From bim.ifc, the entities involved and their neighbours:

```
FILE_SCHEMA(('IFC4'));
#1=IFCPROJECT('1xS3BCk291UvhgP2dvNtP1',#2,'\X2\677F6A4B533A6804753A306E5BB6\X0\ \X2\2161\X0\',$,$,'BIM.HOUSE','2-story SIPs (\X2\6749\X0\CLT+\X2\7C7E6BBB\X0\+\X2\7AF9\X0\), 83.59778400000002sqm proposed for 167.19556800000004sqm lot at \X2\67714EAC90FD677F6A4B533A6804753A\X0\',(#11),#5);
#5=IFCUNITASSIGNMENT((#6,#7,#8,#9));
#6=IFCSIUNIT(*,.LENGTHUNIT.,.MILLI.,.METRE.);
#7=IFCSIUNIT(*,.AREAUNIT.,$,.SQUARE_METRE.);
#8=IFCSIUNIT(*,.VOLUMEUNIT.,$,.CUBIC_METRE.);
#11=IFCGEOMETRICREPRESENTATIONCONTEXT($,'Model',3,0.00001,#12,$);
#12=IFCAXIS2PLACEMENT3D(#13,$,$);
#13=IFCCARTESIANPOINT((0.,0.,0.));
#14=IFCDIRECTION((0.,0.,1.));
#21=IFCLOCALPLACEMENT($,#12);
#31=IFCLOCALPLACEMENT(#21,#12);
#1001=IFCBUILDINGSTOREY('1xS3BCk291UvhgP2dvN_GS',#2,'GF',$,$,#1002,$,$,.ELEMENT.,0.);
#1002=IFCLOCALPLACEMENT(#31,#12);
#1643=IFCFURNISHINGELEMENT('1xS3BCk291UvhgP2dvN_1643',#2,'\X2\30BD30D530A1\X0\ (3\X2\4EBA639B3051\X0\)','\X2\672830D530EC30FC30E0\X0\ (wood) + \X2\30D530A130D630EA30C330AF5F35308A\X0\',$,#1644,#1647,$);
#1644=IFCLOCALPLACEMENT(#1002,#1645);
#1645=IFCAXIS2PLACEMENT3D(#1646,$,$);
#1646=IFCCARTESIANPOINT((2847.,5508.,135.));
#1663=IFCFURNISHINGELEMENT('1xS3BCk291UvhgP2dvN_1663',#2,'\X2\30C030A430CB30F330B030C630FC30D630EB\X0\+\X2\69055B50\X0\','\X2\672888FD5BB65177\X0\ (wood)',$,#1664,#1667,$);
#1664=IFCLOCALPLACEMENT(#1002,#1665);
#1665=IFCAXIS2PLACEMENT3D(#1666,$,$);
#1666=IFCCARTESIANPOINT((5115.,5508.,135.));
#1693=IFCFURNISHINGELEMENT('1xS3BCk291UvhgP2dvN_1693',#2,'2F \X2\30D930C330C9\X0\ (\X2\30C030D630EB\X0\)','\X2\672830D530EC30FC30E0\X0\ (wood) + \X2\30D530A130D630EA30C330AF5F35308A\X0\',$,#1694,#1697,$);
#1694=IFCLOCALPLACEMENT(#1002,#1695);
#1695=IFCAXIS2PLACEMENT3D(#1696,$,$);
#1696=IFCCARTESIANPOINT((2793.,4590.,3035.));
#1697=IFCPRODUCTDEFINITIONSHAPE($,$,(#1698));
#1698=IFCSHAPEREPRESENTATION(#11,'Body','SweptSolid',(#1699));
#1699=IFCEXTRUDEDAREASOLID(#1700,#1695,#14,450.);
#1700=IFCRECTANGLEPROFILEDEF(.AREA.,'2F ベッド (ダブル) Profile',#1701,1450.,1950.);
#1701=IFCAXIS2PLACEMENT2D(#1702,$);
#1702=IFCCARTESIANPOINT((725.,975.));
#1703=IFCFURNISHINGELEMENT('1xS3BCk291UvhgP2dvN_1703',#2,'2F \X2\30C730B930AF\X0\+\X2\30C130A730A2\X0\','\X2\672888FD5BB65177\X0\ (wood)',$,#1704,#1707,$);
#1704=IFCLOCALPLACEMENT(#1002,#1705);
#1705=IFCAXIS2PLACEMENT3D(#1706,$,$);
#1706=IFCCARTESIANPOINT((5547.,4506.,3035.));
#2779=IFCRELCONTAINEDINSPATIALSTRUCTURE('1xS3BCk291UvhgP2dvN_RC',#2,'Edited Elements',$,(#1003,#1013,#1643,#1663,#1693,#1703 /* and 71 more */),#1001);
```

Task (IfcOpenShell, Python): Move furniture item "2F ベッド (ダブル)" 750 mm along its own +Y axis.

```python
import ifcopenshell
import ifcopenshell.api.geometry
import ifcopenshell.util.placement

model = ifcopenshell.open("bim.ifc")

item = model.by_id(1693)
matrix = ifcopenshell.util.placement.get_local_placement(item.ObjectPlacement)
matrix[:3, 3] += matrix[:3, 1] * 750.0
ifcopenshell.api.geometry.edit_object_placement(model, product=item, matrix=matrix, is_si=False)

print(ifcopenshell.util.placement.get_local_placement(item.ObjectPlacement).round(3) + 0.0)

model.write("bim_rev.ifc")
```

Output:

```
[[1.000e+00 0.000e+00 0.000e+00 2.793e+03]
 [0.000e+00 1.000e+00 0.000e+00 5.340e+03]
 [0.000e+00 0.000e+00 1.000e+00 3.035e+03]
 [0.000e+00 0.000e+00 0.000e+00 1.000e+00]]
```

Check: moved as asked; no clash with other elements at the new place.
